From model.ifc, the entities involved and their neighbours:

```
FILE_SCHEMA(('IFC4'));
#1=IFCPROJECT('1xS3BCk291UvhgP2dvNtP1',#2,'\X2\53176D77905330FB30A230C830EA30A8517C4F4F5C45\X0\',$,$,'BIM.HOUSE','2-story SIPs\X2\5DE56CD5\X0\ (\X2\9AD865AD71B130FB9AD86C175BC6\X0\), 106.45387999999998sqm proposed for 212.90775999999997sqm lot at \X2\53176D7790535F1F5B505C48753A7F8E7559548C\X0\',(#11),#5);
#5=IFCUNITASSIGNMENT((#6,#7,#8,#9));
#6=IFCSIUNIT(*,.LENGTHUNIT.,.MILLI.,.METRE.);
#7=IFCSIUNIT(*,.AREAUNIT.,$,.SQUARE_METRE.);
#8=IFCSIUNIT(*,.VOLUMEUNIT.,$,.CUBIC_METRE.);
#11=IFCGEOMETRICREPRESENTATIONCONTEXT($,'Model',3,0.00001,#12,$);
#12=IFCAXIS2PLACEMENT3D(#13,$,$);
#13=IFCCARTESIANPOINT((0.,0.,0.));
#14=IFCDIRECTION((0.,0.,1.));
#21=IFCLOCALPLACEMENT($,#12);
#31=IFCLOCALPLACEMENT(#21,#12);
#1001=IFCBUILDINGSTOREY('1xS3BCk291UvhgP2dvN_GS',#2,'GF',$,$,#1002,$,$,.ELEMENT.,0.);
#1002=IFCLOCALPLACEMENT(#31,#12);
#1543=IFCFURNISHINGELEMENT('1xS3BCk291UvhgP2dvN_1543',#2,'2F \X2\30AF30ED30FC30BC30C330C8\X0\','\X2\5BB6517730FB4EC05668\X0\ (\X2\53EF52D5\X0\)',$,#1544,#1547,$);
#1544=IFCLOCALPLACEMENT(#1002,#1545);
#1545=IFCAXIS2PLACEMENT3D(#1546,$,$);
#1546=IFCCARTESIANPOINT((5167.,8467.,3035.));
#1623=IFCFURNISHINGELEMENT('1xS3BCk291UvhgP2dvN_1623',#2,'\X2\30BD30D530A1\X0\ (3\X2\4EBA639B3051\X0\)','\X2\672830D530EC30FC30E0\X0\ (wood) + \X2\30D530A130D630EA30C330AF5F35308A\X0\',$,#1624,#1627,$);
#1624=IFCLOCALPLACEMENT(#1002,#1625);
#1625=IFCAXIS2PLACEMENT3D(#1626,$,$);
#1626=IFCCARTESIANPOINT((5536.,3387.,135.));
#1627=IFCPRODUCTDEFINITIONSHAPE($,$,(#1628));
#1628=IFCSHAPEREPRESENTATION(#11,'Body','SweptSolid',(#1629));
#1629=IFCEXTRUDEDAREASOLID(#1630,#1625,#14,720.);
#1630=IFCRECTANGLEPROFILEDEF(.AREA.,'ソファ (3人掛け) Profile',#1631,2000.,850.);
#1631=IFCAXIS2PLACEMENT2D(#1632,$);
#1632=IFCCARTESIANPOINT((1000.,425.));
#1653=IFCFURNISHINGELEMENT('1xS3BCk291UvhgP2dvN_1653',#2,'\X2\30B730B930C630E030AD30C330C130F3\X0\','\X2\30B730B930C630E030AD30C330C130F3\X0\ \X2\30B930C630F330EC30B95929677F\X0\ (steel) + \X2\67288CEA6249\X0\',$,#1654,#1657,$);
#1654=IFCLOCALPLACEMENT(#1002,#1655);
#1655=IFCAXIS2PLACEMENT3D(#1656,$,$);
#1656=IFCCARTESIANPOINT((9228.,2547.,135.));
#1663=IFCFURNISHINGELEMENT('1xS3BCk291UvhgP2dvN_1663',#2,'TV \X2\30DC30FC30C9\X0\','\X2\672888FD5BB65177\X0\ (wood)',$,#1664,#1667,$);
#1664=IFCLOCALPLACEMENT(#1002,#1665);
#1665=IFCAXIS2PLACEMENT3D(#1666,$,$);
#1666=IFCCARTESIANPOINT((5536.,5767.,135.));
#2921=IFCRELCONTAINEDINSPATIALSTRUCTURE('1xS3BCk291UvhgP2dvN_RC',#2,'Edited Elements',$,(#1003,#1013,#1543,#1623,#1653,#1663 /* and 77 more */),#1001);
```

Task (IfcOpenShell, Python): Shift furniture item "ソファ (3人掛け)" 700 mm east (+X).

```python
import ifcopenshell
import ifcopenshell.api.geometry
import ifcopenshell.util.placement

model = ifcopenshell.open("model.ifc")

item = model.by_id(1623)
matrix = ifcopenshell.util.placement.get_local_placement(item.ObjectPlacement)
matrix[0, 3] += 700.0
ifcopenshell.api.geometry.edit_object_placement(model, product=item, matrix=matrix, is_si=False)

print(ifcopenshell.util.placement.get_local_placement(item.ObjectPlacement).round(3) + 0.0)

model.write("model_rev.ifc")
```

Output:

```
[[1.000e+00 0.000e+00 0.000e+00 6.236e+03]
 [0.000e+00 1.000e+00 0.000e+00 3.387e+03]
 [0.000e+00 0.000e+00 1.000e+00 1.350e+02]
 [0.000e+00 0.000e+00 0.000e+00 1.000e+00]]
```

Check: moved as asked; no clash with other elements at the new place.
